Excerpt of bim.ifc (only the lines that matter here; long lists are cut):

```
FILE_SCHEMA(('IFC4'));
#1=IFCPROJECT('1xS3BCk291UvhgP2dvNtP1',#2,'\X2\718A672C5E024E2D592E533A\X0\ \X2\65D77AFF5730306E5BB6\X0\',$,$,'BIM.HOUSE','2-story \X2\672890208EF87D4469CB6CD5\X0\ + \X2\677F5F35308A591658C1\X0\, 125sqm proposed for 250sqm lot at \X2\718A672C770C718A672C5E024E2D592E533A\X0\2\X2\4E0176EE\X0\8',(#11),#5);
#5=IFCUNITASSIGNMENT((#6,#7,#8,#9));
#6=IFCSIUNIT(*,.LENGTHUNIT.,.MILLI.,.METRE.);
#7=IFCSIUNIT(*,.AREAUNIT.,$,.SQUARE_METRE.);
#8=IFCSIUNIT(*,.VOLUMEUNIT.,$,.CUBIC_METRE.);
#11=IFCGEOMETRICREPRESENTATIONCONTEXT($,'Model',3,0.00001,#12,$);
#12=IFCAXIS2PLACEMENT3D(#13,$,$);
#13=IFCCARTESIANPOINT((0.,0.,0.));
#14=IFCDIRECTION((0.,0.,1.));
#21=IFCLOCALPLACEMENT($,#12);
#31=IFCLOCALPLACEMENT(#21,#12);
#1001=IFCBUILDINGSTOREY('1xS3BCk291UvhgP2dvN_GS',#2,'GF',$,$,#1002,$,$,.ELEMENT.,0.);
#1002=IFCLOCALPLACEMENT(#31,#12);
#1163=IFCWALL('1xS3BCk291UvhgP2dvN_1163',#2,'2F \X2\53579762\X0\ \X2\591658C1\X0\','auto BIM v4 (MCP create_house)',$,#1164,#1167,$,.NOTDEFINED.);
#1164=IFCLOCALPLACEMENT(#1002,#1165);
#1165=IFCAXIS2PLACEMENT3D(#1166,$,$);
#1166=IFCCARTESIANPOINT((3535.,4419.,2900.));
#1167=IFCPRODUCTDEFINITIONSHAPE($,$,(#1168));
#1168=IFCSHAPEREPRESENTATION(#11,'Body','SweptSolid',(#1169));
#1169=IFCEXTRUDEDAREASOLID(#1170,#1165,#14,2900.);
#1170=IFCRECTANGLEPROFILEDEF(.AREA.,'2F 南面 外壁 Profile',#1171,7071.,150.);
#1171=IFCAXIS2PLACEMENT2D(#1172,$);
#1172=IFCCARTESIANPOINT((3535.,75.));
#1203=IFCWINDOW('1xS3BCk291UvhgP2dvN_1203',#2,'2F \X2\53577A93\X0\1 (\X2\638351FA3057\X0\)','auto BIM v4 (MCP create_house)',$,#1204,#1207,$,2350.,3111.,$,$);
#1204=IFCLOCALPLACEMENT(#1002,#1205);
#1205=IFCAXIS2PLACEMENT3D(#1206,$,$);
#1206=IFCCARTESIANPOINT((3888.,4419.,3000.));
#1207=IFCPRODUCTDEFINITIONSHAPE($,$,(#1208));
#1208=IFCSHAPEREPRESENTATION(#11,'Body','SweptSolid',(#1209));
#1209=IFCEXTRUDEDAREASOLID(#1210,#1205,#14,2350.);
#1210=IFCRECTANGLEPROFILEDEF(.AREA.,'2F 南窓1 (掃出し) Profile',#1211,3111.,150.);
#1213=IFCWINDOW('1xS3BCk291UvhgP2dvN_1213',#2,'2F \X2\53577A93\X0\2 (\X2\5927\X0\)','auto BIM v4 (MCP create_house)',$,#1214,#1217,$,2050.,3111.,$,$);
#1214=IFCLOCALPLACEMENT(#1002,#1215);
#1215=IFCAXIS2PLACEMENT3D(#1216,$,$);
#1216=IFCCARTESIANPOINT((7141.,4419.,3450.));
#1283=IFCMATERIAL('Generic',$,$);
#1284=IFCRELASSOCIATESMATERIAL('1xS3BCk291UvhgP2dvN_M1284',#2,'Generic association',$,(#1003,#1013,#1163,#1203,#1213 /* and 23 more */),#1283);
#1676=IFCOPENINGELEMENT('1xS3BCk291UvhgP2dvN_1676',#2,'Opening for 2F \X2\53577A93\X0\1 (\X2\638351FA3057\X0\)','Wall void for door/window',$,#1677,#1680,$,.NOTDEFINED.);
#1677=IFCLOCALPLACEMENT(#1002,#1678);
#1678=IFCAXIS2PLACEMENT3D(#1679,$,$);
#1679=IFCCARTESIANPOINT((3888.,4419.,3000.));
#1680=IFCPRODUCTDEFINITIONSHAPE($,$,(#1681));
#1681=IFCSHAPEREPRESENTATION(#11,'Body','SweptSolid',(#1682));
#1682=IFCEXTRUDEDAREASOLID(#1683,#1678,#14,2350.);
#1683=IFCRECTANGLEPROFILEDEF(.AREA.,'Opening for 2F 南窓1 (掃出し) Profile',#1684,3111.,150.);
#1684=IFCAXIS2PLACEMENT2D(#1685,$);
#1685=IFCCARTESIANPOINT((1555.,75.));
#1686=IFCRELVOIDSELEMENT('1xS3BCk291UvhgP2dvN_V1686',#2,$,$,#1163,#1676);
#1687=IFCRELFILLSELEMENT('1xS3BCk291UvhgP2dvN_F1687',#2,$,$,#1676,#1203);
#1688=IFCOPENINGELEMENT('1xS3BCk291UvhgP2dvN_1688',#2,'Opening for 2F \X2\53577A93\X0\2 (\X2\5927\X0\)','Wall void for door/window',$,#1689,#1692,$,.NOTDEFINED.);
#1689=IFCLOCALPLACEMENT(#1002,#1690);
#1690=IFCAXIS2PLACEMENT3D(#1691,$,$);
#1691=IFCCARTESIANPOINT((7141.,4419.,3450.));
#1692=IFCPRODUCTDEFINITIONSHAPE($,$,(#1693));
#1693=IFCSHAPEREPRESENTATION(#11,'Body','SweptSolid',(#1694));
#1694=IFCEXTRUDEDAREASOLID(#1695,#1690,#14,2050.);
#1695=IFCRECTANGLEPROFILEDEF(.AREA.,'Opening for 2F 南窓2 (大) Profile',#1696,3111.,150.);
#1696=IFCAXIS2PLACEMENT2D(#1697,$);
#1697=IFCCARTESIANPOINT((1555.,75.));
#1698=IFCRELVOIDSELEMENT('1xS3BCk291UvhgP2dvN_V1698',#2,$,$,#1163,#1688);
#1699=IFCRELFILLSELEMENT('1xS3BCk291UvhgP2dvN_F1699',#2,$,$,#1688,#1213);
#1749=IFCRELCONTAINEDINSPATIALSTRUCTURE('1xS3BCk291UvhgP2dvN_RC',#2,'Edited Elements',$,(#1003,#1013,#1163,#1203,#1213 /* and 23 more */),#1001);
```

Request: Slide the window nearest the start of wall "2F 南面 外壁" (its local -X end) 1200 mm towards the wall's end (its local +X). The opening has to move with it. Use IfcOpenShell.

```python
import ifcopenshell
import ifcopenshell.api.geometry
import ifcopenshell.util.placement
import ifcopenshell.util.unit

model = ifcopenshell.open("bim.ifc")
unit_scale = ifcopenshell.util.unit.calculate_unit_scale(model)

window = model.by_guid("1xS3BCk291UvhgP2dvN_1203")
opening = window.FillsVoids[0].RelatingOpeningElement
wall = opening.VoidsElements[0].RelatingBuildingElement

wall_matrix = ifcopenshell.util.placement.get_local_placement(wall.ObjectPlacement)
shift = wall_matrix[:3, 0] * 1.2 / unit_scale
before = ifcopenshell.util.placement.get_local_placement(window.ObjectPlacement)[:3, 3].copy()

# The window is not placed relative to its opening, so move both.
for product in (opening, window):
    matrix = ifcopenshell.util.placement.get_local_placement(product.ObjectPlacement)
    matrix[:3, 3] += shift
    ifcopenshell.api.geometry.edit_object_placement(model, product=product, matrix=matrix, is_si=False)

after = ifcopenshell.util.placement.get_local_placement(window.ObjectPlacement)[:3, 3]
print("window moved by", (after - before).round(3) + 0.0)

model.write("bim_edited.ifc")
```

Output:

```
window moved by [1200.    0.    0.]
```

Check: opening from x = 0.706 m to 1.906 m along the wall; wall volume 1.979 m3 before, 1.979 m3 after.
